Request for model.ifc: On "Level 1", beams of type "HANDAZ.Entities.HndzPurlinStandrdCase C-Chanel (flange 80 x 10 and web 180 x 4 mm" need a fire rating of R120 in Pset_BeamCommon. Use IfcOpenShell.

First a look at what the model holds.

```python
import ifcopenshell
import ifcopenshell.util.element

model = ifcopenshell.open("model.ifc")
print(model.schema)
storey = next(s for s in model.by_type("IfcBuildingStorey") if s.Name == "Level 1")
beams = [e for e in ifcopenshell.util.element.get_decomposition(storey) if e.is_a("IfcBeam")]
seen = {}
for e in beams:
    element_type = ifcopenshell.util.element.get_type(e)
    key = (element_type.Name if element_type != e and element_type else None, ifcopenshell.util.element.get_pset(e, "Pset_BeamCommon", "FireRating"))
    seen[key] = seen.get(key, 0) + 1
for (name, value), count in sorted(seen.items(), key=str):
    print(count, "x", name, "|", value)
```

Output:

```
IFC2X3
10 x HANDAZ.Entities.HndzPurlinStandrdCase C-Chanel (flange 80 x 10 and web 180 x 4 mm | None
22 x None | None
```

```python
import ifcopenshell
import ifcopenshell.api.pset
import ifcopenshell.util.element

model = ifcopenshell.open("model.ifc")

storey = next(s for s in model.by_type("IfcBuildingStorey") if s.Name == "Level 1")
beams = [e for e in ifcopenshell.util.element.get_decomposition(storey) if e.is_a("IfcBeam")]

count = 0
for e in beams:
    element_type = ifcopenshell.util.element.get_type(e)
    if element_type in (None, e) or element_type.Name != "HANDAZ.Entities.HndzPurlinStandrdCase C-Chanel (flange 80 x 10 and web 180 x 4 mm":
        continue
    # add_pset returns the element's existing set when there is one.
    pset = ifcopenshell.api.pset.add_pset(model, product=e, name="Pset_BeamCommon")
    ifcopenshell.api.pset.edit_pset(model, pset=pset, properties={"FireRating": "R120"})
    count += 1

print(count, "beams updated")

model.write("model_updated.ifc")
```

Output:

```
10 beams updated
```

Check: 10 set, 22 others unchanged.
